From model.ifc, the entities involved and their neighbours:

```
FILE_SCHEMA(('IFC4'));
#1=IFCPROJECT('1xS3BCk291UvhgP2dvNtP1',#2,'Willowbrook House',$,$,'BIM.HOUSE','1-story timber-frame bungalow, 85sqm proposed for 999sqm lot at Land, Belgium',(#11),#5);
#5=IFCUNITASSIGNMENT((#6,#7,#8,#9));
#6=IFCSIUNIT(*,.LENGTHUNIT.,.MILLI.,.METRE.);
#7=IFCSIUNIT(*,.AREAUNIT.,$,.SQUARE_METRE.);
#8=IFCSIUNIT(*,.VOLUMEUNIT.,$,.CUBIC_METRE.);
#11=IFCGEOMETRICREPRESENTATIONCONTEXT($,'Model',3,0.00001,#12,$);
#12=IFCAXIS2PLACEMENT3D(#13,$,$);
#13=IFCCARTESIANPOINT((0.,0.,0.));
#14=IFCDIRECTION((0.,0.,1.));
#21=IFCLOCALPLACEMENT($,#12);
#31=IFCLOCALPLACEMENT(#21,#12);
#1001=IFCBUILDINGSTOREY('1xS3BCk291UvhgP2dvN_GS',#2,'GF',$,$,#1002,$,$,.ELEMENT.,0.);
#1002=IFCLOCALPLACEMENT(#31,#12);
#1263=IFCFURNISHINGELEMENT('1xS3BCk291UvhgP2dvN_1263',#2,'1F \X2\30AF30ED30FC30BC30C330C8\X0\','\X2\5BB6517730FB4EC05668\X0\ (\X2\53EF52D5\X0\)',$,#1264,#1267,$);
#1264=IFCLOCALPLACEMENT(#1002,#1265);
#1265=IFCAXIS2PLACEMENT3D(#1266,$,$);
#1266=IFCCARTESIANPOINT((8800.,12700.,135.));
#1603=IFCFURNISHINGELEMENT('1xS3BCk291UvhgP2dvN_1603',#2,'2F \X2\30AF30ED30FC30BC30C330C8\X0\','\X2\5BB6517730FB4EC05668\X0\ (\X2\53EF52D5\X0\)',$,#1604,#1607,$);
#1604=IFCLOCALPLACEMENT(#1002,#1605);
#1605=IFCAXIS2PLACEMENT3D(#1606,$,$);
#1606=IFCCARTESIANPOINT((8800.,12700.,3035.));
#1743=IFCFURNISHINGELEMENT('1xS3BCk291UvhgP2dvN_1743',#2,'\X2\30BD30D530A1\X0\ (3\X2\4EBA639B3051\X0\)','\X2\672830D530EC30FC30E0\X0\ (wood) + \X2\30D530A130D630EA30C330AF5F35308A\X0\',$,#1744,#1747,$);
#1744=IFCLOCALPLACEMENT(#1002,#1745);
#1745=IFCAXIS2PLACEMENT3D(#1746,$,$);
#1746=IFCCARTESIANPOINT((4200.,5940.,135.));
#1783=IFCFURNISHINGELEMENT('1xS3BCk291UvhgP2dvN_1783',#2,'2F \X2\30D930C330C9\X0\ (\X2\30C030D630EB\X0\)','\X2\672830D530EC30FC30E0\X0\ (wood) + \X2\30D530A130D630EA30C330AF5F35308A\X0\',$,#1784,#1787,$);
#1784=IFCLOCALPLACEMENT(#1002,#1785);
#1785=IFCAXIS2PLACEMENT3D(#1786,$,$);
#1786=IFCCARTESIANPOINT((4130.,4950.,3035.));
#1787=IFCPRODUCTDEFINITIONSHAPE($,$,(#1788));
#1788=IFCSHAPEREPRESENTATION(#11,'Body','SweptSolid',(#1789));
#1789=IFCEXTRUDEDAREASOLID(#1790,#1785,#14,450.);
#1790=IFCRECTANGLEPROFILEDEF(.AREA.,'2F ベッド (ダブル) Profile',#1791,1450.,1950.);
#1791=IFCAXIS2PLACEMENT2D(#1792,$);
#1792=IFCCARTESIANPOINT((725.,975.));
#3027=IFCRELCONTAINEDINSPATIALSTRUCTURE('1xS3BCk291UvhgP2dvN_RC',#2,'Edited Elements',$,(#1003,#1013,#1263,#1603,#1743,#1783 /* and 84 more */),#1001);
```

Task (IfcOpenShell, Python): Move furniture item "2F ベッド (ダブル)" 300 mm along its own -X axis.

```python
import ifcopenshell
import ifcopenshell.api.geometry
import ifcopenshell.util.placement
import ifcopenshell.util.unit

model = ifcopenshell.open("model.ifc")
unit_scale = ifcopenshell.util.unit.calculate_unit_scale(model)

item = model.by_id(1783)
matrix = ifcopenshell.util.placement.get_local_placement(item.ObjectPlacement)
matrix[:3, 3] -= matrix[:3, 0] * 0.3 / unit_scale
ifcopenshell.api.geometry.edit_object_placement(model, product=item, matrix=matrix, is_si=False)

print(ifcopenshell.util.placement.get_local_placement(item.ObjectPlacement).round(3) + 0.0)

model.write("model-out.ifc")
```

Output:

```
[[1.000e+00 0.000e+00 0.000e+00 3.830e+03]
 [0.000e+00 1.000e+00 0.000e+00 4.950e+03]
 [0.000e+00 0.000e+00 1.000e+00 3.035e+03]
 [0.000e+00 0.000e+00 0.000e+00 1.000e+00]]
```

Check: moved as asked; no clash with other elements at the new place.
